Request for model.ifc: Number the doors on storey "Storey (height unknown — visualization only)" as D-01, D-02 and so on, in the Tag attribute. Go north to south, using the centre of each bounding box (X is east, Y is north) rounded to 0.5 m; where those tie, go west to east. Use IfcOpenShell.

First a look at what the model holds.

```python
import ifcopenshell
import ifcopenshell.util.element
import ifcopenshell.util.placement

model = ifcopenshell.open("model.ifc")
print(model.schema)
storey = next(s for s in model.by_type("IfcBuildingStorey") if s.Name == "Storey (height unknown — visualization only)")
doors = [e for e in ifcopenshell.util.element.get_decomposition(storey) if e.is_a("IfcDoor")]
for e in sorted(doors, key=lambda e: e.id()):
    origin = ifcopenshell.util.placement.get_local_placement(e.ObjectPlacement)[:3, 3]
    print(e.id(), e.Tag, e.Name, origin.round(2) + 0.0, sep=" | ")
```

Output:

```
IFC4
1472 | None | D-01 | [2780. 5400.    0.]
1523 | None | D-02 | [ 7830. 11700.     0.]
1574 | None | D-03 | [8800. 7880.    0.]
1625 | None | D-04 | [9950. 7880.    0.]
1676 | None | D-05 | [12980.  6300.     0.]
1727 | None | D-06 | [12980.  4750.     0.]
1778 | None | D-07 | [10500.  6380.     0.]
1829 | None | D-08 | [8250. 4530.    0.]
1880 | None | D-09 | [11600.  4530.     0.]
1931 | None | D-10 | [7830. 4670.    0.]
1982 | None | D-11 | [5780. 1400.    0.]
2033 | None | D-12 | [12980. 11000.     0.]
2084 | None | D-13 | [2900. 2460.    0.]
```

```python
import ifcopenshell
import ifcopenshell.geom
import ifcopenshell.util.element
import ifcopenshell.util.shape

model = ifcopenshell.open("model.ifc")
settings = ifcopenshell.geom.settings()
settings.set("use-world-coords", True)


def centre(element):
    shape = ifcopenshell.geom.create_shape(settings, element)
    return ifcopenshell.util.shape.get_bbox_centroid(shape.geometry)


storey = next(s for s in model.by_type("IfcBuildingStorey") if s.Name == "Storey (height unknown — visualization only)")
doors = [e for e in ifcopenshell.util.element.get_decomposition(storey) if e.is_a("IfcDoor")]

# Insertion points can sit at a corner or the storey origin, so sort by the geometry (in metres).
centres = {e: centre(e) for e in doors}
doors.sort(key=lambda e: (-round(centres[e][1] / 0.5), centres[e][0]))

for i, e in enumerate(doors, start=1):
    number = f"D-{i:02d}"
    e.Tag = number
    print(e.id(), number)

model.write("model-out.ifc")
```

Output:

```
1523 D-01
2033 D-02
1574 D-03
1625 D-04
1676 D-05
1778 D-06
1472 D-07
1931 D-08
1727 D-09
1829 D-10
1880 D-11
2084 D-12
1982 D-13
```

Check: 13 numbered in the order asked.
